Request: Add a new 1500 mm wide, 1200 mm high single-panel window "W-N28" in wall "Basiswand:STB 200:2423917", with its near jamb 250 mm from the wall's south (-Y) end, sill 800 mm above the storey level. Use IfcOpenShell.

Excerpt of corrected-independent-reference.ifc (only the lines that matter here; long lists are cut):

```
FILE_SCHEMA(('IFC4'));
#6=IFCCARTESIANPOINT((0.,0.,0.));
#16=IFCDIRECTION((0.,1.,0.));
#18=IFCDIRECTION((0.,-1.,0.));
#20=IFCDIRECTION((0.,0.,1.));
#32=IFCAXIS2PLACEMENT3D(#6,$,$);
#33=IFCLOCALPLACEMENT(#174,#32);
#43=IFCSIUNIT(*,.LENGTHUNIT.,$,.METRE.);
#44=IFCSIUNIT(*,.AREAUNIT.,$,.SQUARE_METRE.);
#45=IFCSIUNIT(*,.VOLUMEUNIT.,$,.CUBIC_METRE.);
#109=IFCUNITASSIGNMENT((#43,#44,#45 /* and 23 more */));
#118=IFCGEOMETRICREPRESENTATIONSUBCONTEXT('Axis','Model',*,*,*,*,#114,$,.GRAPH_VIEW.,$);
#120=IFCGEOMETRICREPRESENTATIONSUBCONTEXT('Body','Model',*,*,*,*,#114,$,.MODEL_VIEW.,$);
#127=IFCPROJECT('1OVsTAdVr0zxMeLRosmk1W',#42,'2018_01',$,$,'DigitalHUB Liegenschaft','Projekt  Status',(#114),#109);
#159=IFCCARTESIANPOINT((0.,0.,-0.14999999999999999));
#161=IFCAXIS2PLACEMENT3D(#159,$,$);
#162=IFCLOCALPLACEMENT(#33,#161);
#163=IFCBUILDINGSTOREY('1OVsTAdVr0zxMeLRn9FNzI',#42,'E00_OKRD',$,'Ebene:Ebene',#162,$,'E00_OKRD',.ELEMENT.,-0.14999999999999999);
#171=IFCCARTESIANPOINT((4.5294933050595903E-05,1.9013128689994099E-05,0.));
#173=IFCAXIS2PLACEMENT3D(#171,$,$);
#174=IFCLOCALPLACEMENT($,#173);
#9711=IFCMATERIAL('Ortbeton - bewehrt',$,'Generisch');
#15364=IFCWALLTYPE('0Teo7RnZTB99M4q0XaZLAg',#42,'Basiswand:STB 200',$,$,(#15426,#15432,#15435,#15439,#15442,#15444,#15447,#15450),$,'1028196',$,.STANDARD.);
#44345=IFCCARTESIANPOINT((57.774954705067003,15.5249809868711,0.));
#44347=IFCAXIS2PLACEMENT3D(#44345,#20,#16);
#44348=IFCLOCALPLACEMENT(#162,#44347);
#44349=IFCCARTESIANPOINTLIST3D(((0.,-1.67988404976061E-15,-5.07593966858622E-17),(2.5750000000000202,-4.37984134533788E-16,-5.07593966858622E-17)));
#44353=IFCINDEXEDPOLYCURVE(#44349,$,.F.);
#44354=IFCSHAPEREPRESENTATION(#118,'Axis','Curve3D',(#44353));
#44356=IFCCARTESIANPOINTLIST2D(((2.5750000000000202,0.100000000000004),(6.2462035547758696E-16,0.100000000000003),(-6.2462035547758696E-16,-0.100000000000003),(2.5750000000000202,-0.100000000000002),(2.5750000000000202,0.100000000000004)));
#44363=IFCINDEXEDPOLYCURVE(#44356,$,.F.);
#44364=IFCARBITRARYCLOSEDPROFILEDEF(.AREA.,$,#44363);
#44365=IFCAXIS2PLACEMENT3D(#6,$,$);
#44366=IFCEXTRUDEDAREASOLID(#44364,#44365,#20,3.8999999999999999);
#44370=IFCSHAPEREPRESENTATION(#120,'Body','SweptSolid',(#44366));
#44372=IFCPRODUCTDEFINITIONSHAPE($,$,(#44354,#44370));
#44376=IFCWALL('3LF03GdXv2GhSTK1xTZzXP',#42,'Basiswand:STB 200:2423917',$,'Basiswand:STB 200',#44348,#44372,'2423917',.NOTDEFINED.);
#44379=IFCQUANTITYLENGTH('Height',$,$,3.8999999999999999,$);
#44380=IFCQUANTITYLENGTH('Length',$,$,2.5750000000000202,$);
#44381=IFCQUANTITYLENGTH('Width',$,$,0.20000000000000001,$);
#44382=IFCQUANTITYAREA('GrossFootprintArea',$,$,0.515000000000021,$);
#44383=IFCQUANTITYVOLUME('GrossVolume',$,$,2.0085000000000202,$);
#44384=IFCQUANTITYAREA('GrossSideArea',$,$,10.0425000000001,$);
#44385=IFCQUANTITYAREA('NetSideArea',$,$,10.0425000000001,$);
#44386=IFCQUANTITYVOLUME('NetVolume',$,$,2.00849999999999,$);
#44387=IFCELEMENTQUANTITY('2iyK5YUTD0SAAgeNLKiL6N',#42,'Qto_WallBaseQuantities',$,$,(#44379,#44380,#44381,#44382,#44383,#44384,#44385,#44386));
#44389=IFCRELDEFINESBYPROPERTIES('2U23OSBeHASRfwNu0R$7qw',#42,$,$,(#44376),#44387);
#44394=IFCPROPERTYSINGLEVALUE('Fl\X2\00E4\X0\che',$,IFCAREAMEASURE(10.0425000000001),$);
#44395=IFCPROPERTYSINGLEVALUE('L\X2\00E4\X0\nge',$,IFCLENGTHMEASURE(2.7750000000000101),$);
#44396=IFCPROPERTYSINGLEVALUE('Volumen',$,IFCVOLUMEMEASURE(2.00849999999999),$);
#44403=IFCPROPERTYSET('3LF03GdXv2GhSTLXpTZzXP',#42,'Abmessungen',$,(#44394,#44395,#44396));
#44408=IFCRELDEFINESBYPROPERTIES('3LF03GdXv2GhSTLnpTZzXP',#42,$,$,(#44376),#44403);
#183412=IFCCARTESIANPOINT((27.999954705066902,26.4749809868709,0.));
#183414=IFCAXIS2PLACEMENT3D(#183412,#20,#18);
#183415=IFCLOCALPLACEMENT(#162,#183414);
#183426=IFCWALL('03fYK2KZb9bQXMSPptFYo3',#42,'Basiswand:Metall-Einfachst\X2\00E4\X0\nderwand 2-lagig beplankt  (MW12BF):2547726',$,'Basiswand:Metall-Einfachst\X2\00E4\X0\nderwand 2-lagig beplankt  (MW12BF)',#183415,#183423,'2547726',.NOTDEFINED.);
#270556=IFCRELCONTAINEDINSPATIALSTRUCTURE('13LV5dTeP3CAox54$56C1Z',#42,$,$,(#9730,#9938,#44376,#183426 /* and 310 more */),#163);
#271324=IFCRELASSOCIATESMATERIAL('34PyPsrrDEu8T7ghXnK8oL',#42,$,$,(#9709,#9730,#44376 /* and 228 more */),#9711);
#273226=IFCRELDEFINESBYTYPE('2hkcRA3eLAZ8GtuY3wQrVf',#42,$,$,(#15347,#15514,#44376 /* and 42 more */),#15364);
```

```python
import numpy as np
import ifcopenshell
import ifcopenshell.api.feature
import ifcopenshell.api.geometry
import ifcopenshell.api.pset
import ifcopenshell.api.root
import ifcopenshell.api.spatial
import ifcopenshell.geom
import ifcopenshell.util.element
import ifcopenshell.util.placement
import ifcopenshell.util.representation
import ifcopenshell.util.shape
import ifcopenshell.util.unit

model = ifcopenshell.open("corrected-independent-reference.ifc")
unit_scale = ifcopenshell.util.unit.calculate_unit_scale(model)
area_scale = ifcopenshell.util.unit.calculate_unit_scale(model, "AREAUNIT")
volume_scale = ifcopenshell.util.unit.calculate_unit_scale(model, "VOLUMEUNIT")
settings = ifcopenshell.geom.settings()


def volume(element):
    """Net volume in cubic metres, openings subtracted."""
    shape = ifcopenshell.geom.create_shape(settings, element)
    return ifcopenshell.util.shape.get_volume(shape.geometry)


wall = model.by_guid("3LF03GdXv2GhSTK1xTZzXP")
storey = ifcopenshell.util.element.get_container(wall, ifc_class="IfcBuildingStorey")
context = ifcopenshell.util.representation.get_context(model, "Model", "Body", "MODEL_VIEW")
before = volume(wall)

width, height, from_end, sill = 1.5, 1.2, 0.25, 0.8  # metres

# The wall runs along its own X axis, and the end named is its -X end.
wall_shape = ifcopenshell.geom.create_shape(settings, wall)
x, y, z = ifcopenshell.util.shape.get_vertices(wall_shape.geometry).T
start = x.min() + from_end
face, thickness = float(y.min()), float(y.max() - y.min())
wall_matrix = ifcopenshell.util.placement.get_local_placement(wall.ObjectPlacement)
level = ifcopenshell.util.placement.get_local_placement(storey.ObjectPlacement)[2, 3]


def in_wall(x, y):
    """Placement at x, y metres in the wall's axes, at sill height."""
    matrix = wall_matrix.copy()
    matrix[:, 3] = wall_matrix @ np.array([x / unit_scale, y / unit_scale, 0.0, 1.0])
    matrix[2, 3] = level + sill / unit_scale
    return matrix


# Opening: a box that overshoots both wall faces by 50 mm.
opening = ifcopenshell.api.root.create_entity(model, ifc_class="IfcOpeningElement", predefined_type="OPENING")
box = ifcopenshell.api.geometry.add_wall_representation(
    model, context=context, length=width, height=height, thickness=thickness + 0.1
)
ifcopenshell.api.geometry.assign_representation(model, product=opening, representation=box)
ifcopenshell.api.geometry.edit_object_placement(model, product=opening, matrix=in_wall(start, face - 0.05), is_si=False)
ifcopenshell.api.feature.add_feature(model, feature=opening, element=wall)

window = ifcopenshell.api.root.create_entity(model, ifc_class="IfcWindow", name="W-N28", predefined_type="WINDOW")
window.OverallWidth, window.OverallHeight = width / unit_scale, height / unit_scale
window.PartitioningType = "SINGLE_PANEL"
body = ifcopenshell.api.geometry.add_window_representation(
    model,
    context=context,
    overall_width=window.OverallWidth,
    overall_height=window.OverallHeight,
    partition_type="SINGLE_PANEL",
)
ifcopenshell.api.geometry.assign_representation(model, product=window, representation=body)
ifcopenshell.api.spatial.assign_container(model, products=[window], relating_structure=storey)
ifcopenshell.api.feature.add_filling(model, opening=opening, element=window)

# Centre the window in the wall's thickness.
ifcopenshell.api.geometry.edit_object_placement(model, product=window, matrix=in_wall(start, face), is_si=False)
window_shape = ifcopenshell.geom.create_shape(settings, window)
depth = ifcopenshell.util.shape.get_vertices(window_shape.geometry)[:, 1]
offset = face + thickness / 2 - (depth.min() + depth.max()) / 2
ifcopenshell.api.geometry.edit_object_placement(model, product=window, matrix=in_wall(start, offset), is_si=False)

after = volume(wall)

# Update the wall's stored quantities.
qto = model.by_id(ifcopenshell.util.element.get_pset(wall, "Qto_WallBaseQuantities", should_inherit=False)["id"])
ifcopenshell.api.pset.edit_qto(model, qto=qto, properties={
    "NetSideArea": after / thickness / area_scale,
    "NetVolume": after / volume_scale,
})
pset = model.by_id(ifcopenshell.util.element.get_pset(wall, "Abmessungen", should_inherit=False)["id"])
ifcopenshell.api.pset.edit_pset(model, pset=pset, properties={
    "Fläche": model.create_entity("IfcAreaMeasure", after / thickness / area_scale),
    "Volumen": model.create_entity("IfcVolumeMeasure", after / volume_scale),
})

print(f"wall volume {before:.3f} -> {after:.3f} m3")

model.write("corrected-independent-reference_rev.ifc")
```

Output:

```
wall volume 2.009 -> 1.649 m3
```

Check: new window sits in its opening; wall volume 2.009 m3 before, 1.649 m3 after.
